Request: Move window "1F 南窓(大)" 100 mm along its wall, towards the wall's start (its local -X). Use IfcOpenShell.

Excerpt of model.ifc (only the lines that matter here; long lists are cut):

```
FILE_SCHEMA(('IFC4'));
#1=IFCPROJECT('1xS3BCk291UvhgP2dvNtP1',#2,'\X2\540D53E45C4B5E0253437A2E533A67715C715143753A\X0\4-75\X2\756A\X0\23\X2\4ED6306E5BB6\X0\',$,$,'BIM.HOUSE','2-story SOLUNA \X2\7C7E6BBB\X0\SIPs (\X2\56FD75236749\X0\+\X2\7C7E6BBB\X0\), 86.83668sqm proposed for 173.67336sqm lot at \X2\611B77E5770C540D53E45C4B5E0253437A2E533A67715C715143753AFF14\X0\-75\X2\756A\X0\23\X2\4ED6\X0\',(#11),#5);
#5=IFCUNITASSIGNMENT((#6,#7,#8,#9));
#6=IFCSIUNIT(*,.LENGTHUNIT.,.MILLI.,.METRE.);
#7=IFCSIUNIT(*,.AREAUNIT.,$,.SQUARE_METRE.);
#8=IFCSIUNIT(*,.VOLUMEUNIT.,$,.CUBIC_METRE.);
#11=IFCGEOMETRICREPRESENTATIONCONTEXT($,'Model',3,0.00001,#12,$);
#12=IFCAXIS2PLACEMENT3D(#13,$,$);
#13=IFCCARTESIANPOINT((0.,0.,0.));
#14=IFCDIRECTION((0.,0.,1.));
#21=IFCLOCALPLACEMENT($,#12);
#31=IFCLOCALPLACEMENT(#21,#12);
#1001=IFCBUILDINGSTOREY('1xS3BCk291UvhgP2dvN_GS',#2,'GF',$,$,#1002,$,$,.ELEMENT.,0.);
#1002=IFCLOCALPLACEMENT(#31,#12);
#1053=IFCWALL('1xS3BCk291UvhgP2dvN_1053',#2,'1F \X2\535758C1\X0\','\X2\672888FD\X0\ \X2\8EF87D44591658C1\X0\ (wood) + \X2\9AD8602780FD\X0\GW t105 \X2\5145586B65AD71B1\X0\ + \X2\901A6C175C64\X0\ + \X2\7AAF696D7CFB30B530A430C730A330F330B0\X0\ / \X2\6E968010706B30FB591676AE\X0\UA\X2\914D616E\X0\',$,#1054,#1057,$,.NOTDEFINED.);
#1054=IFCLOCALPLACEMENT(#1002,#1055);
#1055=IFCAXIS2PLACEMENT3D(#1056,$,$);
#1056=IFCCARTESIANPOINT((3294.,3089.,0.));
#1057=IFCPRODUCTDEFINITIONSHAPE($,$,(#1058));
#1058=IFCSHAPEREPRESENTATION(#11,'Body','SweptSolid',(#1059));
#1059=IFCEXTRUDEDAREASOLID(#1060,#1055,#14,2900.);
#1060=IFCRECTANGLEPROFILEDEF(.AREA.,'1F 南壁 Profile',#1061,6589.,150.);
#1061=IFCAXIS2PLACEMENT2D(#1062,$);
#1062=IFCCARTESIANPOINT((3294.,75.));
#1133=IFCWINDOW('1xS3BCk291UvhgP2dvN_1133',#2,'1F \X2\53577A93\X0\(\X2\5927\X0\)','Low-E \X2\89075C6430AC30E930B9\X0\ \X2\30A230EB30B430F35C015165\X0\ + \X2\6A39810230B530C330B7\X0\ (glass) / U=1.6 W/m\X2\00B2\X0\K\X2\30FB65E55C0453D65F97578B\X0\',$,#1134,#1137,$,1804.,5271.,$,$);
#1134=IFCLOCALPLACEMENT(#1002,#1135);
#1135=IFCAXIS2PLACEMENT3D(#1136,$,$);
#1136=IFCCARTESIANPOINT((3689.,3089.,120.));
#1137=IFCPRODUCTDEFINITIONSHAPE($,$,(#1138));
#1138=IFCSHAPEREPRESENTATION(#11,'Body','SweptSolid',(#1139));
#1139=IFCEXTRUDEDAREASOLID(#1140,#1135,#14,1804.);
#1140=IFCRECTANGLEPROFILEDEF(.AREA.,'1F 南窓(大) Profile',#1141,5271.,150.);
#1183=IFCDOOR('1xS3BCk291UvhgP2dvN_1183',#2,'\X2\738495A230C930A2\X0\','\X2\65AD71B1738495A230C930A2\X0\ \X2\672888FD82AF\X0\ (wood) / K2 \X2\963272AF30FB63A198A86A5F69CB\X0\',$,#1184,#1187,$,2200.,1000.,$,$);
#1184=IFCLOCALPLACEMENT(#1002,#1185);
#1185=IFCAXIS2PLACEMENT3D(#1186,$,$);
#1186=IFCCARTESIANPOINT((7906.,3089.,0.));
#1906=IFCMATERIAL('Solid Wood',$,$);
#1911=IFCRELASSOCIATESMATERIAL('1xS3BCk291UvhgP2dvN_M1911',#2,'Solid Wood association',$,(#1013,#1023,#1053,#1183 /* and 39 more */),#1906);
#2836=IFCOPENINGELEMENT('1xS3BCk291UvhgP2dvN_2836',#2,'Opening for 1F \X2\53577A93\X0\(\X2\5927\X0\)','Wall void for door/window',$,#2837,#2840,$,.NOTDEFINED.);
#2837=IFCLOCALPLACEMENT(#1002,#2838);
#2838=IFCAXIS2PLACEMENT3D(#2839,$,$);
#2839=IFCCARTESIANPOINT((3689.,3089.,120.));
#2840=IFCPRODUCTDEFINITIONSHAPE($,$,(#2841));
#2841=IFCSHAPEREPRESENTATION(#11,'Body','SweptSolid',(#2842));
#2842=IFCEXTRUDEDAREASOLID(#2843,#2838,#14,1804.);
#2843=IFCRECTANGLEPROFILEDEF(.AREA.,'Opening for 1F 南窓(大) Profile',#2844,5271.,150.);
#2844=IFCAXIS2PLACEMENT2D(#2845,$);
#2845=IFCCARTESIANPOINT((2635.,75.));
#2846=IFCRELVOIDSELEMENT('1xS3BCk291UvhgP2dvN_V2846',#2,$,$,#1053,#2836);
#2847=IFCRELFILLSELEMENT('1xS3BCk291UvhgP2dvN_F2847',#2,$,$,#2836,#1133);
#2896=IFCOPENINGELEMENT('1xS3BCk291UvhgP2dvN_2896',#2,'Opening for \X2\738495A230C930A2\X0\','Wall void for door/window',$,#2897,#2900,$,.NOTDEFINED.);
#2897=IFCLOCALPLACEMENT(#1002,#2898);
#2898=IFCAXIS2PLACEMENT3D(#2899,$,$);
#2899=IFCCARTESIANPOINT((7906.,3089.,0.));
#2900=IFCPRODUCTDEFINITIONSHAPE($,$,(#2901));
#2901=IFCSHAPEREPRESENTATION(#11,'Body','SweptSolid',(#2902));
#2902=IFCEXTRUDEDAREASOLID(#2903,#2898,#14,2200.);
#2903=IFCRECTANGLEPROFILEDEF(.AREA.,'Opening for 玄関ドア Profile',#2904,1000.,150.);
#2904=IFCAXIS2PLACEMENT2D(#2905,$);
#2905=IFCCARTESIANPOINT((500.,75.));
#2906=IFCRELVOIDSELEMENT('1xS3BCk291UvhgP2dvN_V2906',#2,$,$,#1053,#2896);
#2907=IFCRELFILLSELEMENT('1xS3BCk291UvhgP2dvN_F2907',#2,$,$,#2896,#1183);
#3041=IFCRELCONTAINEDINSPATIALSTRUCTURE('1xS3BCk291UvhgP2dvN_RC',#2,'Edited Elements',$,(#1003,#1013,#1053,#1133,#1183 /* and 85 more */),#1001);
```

```python
import ifcopenshell
import ifcopenshell.api.geometry
import ifcopenshell.util.placement

model = ifcopenshell.open("model.ifc")

window = model.by_id(1133)
opening = window.FillsVoids[0].RelatingOpeningElement
wall = opening.VoidsElements[0].RelatingBuildingElement

wall_matrix = ifcopenshell.util.placement.get_local_placement(wall.ObjectPlacement)
shift = wall_matrix[:3, 0] * -100.0
before = ifcopenshell.util.placement.get_local_placement(window.ObjectPlacement)[:3, 3].copy()

# The window is not placed relative to its opening, so move both.
for product in (opening, window):
    matrix = ifcopenshell.util.placement.get_local_placement(product.ObjectPlacement)
    matrix[:3, 3] += shift
    ifcopenshell.api.geometry.edit_object_placement(model, product=product, matrix=matrix, is_si=False)

after = ifcopenshell.util.placement.get_local_placement(window.ObjectPlacement)[:3, 3]
print("window moved by", (after - before).round(3) + 0.0)

model.write("model_v2.ifc")
```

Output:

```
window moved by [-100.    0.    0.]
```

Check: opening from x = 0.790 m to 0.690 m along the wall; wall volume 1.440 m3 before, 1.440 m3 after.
